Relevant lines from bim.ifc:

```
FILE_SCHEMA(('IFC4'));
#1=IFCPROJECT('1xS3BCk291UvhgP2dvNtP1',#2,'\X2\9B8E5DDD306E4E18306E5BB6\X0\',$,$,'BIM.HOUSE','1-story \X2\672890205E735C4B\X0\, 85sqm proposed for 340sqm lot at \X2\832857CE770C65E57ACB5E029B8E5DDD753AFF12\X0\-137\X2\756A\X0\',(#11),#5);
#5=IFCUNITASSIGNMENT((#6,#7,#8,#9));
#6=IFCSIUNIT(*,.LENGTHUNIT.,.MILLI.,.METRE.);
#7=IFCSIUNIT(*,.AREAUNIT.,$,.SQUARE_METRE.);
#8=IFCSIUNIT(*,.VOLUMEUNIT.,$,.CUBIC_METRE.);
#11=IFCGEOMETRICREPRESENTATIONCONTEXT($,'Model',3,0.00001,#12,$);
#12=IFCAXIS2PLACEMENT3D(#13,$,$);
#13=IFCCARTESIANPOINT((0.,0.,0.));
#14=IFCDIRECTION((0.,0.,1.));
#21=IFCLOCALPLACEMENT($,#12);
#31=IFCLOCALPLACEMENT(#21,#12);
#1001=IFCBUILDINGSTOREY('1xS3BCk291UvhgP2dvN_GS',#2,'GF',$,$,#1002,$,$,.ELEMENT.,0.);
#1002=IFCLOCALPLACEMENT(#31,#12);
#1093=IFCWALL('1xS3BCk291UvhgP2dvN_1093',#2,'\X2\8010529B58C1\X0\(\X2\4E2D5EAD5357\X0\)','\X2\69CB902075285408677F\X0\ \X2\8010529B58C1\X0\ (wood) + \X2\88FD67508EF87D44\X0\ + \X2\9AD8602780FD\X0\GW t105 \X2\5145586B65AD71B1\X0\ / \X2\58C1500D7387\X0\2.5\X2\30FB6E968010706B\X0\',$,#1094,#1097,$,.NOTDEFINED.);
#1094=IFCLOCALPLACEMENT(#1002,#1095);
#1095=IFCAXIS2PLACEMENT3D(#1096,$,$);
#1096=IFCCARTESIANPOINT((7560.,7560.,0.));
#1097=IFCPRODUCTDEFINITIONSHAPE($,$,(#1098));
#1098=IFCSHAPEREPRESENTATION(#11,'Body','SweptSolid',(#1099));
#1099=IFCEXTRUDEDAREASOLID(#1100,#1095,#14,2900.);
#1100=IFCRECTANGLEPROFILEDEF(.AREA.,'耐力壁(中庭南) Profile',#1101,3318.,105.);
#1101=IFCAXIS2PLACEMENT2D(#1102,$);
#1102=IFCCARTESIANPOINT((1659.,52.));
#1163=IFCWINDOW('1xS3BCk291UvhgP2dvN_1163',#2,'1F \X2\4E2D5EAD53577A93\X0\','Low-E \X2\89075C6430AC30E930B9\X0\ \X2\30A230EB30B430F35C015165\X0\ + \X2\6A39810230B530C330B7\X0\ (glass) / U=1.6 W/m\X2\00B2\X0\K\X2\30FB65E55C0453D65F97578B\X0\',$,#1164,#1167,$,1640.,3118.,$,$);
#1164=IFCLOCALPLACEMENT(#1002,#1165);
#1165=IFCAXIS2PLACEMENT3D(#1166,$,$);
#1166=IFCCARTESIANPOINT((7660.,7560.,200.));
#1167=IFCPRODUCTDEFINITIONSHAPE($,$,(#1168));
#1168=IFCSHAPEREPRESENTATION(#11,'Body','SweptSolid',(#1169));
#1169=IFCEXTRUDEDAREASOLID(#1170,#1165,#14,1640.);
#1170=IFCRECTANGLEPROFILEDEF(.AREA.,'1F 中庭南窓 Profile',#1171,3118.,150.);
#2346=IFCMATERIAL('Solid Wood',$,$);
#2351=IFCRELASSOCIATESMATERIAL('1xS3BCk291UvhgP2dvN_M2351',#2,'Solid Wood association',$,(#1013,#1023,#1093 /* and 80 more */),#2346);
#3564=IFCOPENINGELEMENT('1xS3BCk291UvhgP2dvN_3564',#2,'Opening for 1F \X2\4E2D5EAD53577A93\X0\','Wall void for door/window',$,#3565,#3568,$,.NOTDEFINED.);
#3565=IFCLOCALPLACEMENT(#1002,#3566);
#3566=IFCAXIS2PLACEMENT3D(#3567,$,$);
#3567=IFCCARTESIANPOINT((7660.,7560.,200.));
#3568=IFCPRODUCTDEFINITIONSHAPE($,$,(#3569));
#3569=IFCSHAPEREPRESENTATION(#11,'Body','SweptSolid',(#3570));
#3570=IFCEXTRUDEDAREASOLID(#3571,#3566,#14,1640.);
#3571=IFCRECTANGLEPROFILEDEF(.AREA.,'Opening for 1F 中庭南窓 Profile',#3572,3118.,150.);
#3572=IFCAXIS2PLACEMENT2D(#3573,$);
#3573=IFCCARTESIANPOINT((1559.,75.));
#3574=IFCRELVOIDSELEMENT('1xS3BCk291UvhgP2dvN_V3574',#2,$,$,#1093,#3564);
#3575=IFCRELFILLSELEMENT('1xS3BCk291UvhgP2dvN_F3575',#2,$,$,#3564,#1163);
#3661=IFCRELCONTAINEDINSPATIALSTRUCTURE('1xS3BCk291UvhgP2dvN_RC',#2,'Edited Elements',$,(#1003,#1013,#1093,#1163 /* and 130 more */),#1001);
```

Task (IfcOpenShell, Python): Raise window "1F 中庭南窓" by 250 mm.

```python
import numpy as np
import ifcopenshell
import ifcopenshell.api.geometry
import ifcopenshell.util.placement
import ifcopenshell.util.unit

model = ifcopenshell.open("bim.ifc")
unit_scale = ifcopenshell.util.unit.calculate_unit_scale(model)

window = model.by_guid("1xS3BCk291UvhgP2dvN_1163")
opening = window.FillsVoids[0].RelatingOpeningElement
dz = 250.0

shift = np.array([0.0, 0.0, dz])
# The window is not placed relative to its opening, so move both.
for product in (opening, window):
    matrix = ifcopenshell.util.placement.get_local_placement(product.ObjectPlacement)
    matrix[:3, 3] += shift
    ifcopenshell.api.geometry.edit_object_placement(model, product=product, matrix=matrix, is_si=False)

print(f"moved by {dz * unit_scale:+.3f} m")

model.write("bim-out.ifc")
```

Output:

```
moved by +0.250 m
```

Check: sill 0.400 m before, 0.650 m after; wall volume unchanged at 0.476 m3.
